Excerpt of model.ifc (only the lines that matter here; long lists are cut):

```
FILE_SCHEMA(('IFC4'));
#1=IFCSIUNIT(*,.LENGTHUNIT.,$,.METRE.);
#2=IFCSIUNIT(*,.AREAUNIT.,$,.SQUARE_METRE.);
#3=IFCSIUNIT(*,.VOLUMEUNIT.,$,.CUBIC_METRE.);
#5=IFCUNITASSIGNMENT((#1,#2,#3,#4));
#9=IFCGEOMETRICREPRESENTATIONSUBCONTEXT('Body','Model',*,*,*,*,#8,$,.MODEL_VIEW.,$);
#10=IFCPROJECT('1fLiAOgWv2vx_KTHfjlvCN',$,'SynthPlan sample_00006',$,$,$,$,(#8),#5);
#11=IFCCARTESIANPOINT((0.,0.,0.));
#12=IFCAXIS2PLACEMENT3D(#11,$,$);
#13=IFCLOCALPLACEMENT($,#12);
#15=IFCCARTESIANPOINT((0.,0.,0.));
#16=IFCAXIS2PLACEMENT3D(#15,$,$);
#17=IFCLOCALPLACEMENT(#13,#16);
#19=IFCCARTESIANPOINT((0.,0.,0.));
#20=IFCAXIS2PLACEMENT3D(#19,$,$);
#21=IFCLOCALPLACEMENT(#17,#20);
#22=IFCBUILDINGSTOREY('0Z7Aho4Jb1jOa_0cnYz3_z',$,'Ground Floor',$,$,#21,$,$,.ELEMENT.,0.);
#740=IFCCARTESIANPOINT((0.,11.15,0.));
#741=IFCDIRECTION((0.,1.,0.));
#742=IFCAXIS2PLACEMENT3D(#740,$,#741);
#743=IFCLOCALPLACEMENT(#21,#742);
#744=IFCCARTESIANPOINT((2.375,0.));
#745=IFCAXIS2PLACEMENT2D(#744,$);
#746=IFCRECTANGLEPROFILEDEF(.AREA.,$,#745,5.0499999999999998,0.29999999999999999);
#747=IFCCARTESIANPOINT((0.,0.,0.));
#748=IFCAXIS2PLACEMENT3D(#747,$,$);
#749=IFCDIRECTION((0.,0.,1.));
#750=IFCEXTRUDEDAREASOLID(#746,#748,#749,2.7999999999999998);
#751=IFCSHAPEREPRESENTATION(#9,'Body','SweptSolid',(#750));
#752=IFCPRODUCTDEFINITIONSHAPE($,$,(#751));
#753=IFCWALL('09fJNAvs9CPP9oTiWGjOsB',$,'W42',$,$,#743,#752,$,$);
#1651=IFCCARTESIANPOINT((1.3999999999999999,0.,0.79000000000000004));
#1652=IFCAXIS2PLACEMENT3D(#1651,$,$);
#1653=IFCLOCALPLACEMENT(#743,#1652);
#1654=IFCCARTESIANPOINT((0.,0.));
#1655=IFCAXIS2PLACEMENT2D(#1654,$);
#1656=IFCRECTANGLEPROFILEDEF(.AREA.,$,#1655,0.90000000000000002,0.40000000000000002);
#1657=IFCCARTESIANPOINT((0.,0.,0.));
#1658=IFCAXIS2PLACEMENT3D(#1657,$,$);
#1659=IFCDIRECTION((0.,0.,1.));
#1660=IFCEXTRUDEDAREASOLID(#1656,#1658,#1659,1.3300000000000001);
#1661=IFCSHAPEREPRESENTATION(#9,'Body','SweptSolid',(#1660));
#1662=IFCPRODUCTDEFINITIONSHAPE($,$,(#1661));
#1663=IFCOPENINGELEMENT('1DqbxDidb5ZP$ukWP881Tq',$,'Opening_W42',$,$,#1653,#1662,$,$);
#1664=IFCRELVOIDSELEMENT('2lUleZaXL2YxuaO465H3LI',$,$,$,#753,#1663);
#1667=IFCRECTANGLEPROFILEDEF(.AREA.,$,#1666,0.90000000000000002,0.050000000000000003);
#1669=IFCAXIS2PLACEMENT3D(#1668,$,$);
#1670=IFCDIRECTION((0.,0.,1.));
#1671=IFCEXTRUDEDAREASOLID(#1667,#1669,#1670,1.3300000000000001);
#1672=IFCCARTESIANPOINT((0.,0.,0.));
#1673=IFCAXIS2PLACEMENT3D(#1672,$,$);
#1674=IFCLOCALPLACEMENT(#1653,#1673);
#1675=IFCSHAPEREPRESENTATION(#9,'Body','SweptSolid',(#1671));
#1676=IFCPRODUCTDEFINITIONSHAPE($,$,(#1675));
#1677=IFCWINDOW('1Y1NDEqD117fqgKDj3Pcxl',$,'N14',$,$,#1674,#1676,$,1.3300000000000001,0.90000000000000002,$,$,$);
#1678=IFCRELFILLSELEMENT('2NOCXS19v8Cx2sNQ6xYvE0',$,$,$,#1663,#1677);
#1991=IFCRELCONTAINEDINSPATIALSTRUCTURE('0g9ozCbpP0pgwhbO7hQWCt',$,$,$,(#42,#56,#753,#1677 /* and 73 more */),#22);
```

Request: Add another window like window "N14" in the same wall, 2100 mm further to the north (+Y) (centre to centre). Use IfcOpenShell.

```python
import ifcopenshell
import ifcopenshell.api.feature
import ifcopenshell.api.geometry
import ifcopenshell.api.root
import ifcopenshell.geom
import ifcopenshell.util.element
import ifcopenshell.util.placement
import ifcopenshell.util.shape
import ifcopenshell.util.unit

model = ifcopenshell.open("model.ifc")
unit_scale = ifcopenshell.util.unit.calculate_unit_scale(model)
settings = ifcopenshell.geom.settings()


def volume(element):
    """Net volume in cubic metres, openings subtracted."""
    shape = ifcopenshell.geom.create_shape(settings, element)
    return ifcopenshell.util.shape.get_volume(shape.geometry)


window = model.by_guid("1Y1NDEqD117fqgKDj3Pcxl")
opening = window.FillsVoids[0].RelatingOpeningElement
wall = opening.VoidsElements[0].RelatingBuildingElement
before = volume(wall)
shift = ifcopenshell.util.placement.get_local_placement(wall.ObjectPlacement)[:3, 0] * 2.1 / unit_scale

# copy_class copies the void relationship, type, container and properties, but no geometry.
new_opening = ifcopenshell.api.root.copy_class(model, product=opening)
new_opening.Representation = ifcopenshell.util.element.copy_deep(
    model, opening.Representation, exclude=["IfcGeometricRepresentationContext", "IfcRepresentationMap"]
)
new_window = ifcopenshell.api.root.copy_class(model, product=window)
new_window.Representation = ifcopenshell.util.element.copy_deep(
    model, window.Representation, exclude=["IfcGeometricRepresentationContext", "IfcRepresentationMap"]
)
ifcopenshell.api.feature.add_filling(model, opening=new_opening, element=new_window)

for old, new in ((opening, new_opening), (window, new_window)):
    matrix = ifcopenshell.util.placement.get_local_placement(old.ObjectPlacement)
    matrix[:3, 3] += shift
    ifcopenshell.api.geometry.edit_object_placement(model, product=new, matrix=matrix, is_si=False)

after = volume(wall)

print(f"wall volume {before:.3f} -> {after:.3f} m3")

model.write("model_rev.ifc")
```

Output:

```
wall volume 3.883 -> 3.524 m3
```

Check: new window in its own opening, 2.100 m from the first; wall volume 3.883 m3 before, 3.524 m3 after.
